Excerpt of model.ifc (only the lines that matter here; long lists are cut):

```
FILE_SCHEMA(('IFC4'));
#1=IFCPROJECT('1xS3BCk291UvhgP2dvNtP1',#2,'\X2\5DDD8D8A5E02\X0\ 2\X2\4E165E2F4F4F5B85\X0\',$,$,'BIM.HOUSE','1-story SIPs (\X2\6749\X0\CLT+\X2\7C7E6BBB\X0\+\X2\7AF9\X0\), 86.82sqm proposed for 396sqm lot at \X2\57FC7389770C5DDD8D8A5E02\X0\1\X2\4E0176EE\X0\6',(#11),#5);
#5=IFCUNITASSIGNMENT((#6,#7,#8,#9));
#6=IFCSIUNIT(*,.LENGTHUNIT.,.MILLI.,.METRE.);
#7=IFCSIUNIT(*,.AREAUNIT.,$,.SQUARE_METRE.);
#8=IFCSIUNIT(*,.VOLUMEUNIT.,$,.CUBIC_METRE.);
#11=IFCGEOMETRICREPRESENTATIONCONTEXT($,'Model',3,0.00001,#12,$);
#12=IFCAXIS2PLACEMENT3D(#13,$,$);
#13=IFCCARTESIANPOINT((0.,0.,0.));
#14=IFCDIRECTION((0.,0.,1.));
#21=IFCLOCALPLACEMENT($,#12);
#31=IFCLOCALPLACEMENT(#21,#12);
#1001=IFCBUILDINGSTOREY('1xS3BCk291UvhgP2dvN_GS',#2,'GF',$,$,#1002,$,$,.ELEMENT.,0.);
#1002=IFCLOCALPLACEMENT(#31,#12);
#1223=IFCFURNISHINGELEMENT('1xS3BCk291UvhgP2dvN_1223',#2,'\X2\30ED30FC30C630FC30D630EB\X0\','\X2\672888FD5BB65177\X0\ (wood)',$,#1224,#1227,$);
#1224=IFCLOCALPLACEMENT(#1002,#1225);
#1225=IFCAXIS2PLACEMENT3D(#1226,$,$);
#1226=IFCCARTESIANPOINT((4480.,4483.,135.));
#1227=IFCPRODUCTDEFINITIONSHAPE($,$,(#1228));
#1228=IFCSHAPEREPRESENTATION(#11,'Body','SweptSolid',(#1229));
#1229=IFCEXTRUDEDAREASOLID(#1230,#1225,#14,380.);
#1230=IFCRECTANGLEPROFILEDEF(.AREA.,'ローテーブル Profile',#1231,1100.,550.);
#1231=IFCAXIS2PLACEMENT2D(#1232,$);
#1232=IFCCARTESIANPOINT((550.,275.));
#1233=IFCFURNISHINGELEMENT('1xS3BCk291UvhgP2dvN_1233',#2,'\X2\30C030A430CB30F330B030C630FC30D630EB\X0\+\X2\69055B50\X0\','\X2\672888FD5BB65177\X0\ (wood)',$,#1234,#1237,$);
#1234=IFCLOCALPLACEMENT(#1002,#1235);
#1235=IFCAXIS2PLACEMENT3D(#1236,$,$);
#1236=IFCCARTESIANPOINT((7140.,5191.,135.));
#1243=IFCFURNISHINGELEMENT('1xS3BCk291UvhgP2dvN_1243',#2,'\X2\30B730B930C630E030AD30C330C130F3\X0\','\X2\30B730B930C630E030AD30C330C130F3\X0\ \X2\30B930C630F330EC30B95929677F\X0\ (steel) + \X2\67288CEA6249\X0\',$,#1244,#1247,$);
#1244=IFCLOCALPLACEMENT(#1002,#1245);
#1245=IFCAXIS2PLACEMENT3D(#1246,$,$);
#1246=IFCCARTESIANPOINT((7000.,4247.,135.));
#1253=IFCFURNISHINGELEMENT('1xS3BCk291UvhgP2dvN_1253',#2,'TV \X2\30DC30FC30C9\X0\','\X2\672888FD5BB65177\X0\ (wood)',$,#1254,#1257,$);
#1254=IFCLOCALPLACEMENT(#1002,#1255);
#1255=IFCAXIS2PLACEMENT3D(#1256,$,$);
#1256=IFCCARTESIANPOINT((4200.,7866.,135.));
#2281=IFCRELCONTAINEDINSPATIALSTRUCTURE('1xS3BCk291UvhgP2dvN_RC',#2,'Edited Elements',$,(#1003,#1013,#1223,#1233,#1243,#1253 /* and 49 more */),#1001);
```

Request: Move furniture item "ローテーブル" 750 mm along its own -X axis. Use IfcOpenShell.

```python
import ifcopenshell
import ifcopenshell.api.geometry
import ifcopenshell.util.placement
import ifcopenshell.util.unit

model = ifcopenshell.open("model.ifc")
unit_scale = ifcopenshell.util.unit.calculate_unit_scale(model)

item = model.by_guid("1xS3BCk291UvhgP2dvN_1223")
matrix = ifcopenshell.util.placement.get_local_placement(item.ObjectPlacement)
matrix[:3, 3] -= matrix[:3, 0] * 0.75 / unit_scale
ifcopenshell.api.geometry.edit_object_placement(model, product=item, matrix=matrix, is_si=False)

print(ifcopenshell.util.placement.get_local_placement(item.ObjectPlacement).round(3) + 0.0)

model.write("model_rev.ifc")
```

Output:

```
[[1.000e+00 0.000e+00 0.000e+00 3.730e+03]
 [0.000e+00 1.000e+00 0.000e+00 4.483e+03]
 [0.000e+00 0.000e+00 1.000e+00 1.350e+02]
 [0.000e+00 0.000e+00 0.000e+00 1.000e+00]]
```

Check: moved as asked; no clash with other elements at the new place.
